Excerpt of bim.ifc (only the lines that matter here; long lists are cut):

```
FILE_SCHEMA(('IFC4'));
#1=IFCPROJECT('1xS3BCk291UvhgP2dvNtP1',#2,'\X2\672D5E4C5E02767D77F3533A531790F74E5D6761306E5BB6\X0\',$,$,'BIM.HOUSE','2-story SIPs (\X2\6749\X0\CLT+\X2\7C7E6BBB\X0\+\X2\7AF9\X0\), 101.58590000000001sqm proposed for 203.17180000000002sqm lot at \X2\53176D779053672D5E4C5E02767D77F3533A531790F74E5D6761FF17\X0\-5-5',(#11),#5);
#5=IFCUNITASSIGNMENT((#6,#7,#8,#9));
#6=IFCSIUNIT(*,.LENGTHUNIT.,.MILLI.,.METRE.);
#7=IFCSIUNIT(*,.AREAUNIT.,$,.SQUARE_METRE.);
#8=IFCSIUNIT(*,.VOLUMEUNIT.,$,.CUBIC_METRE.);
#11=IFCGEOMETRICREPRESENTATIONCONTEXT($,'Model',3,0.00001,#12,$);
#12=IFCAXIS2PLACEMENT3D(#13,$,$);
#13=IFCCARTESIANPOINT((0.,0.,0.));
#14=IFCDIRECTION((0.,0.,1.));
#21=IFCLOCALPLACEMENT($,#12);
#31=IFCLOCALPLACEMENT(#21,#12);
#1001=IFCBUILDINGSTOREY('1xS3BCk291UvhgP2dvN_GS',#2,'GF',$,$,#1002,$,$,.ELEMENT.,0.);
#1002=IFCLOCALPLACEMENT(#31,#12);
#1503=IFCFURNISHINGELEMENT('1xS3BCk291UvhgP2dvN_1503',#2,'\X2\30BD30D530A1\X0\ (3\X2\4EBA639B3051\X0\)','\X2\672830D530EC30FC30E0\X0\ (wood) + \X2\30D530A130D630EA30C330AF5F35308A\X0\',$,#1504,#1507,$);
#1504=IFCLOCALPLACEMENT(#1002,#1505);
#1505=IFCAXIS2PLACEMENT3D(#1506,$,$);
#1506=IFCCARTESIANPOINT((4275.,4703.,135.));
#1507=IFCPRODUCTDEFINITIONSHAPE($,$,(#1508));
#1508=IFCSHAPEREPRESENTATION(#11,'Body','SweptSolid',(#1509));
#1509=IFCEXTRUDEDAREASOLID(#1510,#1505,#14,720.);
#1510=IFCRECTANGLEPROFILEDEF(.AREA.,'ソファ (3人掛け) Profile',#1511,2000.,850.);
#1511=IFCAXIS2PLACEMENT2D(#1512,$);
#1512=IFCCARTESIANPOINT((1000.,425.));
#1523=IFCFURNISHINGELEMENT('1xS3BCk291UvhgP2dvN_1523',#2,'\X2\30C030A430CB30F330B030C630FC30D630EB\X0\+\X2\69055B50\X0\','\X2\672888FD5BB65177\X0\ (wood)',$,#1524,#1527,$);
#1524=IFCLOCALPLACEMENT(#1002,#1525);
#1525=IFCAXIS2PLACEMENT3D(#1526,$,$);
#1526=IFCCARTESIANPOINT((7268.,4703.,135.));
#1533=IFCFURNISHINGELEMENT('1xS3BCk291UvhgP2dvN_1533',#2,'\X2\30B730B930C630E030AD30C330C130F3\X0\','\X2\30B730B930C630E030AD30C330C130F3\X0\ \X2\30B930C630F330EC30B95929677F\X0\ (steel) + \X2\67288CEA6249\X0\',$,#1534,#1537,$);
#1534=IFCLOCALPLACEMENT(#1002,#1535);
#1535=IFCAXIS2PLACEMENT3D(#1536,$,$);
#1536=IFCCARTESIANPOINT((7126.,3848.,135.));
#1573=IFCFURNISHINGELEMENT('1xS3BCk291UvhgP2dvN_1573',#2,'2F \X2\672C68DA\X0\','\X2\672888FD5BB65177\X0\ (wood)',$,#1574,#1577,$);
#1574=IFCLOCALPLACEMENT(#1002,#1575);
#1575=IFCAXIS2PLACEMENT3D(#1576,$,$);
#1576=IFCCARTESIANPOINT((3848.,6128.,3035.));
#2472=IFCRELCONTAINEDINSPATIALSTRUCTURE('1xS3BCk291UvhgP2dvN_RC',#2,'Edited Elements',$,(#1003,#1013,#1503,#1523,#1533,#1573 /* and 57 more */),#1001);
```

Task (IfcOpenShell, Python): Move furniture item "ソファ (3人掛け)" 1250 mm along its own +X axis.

```python
import ifcopenshell
import ifcopenshell.api.geometry
import ifcopenshell.util.placement
import ifcopenshell.util.unit

model = ifcopenshell.open("bim.ifc")
unit_scale = ifcopenshell.util.unit.calculate_unit_scale(model)

item = model.by_guid("1xS3BCk291UvhgP2dvN_1503")
matrix = ifcopenshell.util.placement.get_local_placement(item.ObjectPlacement)
matrix[:3, 3] += matrix[:3, 0] * 1.25 / unit_scale
ifcopenshell.api.geometry.edit_object_placement(model, product=item, matrix=matrix, is_si=False)

print(ifcopenshell.util.placement.get_local_placement(item.ObjectPlacement).round(3) + 0.0)

model.write("bim_updated.ifc")
```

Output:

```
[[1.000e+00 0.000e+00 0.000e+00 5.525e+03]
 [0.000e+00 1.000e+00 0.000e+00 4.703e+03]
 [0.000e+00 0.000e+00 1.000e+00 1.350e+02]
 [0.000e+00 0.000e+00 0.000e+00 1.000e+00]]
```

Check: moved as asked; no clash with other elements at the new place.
